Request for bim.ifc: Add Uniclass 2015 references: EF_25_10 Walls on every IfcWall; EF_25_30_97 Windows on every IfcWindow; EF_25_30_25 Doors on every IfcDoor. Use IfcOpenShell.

First a look at what the model holds.

```python
import ifcopenshell

model = ifcopenshell.open("bim.ifc")
print(model.schema)
print("classifications:", [c.Name for c in model.by_type("IfcClassification")])
for ifc_class in ("IfcDoor", "IfcRoof", "IfcStair", "IfcWall", "IfcWindow"):
    print(ifc_class, len(model.by_type(ifc_class)))
```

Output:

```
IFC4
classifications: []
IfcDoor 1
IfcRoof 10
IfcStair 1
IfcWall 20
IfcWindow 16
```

```python
import ifcopenshell
import ifcopenshell.api.classification

model = ifcopenshell.open("bim.ifc")

system = ifcopenshell.api.classification.add_classification(model, classification="Uniclass 2015")

codes = {
    "IfcWall": ("EF_25_10", "Walls"),
    "IfcWindow": ("EF_25_30_97", "Windows"),
    "IfcDoor": ("EF_25_30_25", "Doors"),
}
for ifc_class, (code, name) in codes.items():
    products = model.by_type(ifc_class)
    ifcopenshell.api.classification.add_reference(
        model, products=products, classification=system, identification=code, name=name
    )
    print(code, len(products))

model.write("bim_edited.ifc")
```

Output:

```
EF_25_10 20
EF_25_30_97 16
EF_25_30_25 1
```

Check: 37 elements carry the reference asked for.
